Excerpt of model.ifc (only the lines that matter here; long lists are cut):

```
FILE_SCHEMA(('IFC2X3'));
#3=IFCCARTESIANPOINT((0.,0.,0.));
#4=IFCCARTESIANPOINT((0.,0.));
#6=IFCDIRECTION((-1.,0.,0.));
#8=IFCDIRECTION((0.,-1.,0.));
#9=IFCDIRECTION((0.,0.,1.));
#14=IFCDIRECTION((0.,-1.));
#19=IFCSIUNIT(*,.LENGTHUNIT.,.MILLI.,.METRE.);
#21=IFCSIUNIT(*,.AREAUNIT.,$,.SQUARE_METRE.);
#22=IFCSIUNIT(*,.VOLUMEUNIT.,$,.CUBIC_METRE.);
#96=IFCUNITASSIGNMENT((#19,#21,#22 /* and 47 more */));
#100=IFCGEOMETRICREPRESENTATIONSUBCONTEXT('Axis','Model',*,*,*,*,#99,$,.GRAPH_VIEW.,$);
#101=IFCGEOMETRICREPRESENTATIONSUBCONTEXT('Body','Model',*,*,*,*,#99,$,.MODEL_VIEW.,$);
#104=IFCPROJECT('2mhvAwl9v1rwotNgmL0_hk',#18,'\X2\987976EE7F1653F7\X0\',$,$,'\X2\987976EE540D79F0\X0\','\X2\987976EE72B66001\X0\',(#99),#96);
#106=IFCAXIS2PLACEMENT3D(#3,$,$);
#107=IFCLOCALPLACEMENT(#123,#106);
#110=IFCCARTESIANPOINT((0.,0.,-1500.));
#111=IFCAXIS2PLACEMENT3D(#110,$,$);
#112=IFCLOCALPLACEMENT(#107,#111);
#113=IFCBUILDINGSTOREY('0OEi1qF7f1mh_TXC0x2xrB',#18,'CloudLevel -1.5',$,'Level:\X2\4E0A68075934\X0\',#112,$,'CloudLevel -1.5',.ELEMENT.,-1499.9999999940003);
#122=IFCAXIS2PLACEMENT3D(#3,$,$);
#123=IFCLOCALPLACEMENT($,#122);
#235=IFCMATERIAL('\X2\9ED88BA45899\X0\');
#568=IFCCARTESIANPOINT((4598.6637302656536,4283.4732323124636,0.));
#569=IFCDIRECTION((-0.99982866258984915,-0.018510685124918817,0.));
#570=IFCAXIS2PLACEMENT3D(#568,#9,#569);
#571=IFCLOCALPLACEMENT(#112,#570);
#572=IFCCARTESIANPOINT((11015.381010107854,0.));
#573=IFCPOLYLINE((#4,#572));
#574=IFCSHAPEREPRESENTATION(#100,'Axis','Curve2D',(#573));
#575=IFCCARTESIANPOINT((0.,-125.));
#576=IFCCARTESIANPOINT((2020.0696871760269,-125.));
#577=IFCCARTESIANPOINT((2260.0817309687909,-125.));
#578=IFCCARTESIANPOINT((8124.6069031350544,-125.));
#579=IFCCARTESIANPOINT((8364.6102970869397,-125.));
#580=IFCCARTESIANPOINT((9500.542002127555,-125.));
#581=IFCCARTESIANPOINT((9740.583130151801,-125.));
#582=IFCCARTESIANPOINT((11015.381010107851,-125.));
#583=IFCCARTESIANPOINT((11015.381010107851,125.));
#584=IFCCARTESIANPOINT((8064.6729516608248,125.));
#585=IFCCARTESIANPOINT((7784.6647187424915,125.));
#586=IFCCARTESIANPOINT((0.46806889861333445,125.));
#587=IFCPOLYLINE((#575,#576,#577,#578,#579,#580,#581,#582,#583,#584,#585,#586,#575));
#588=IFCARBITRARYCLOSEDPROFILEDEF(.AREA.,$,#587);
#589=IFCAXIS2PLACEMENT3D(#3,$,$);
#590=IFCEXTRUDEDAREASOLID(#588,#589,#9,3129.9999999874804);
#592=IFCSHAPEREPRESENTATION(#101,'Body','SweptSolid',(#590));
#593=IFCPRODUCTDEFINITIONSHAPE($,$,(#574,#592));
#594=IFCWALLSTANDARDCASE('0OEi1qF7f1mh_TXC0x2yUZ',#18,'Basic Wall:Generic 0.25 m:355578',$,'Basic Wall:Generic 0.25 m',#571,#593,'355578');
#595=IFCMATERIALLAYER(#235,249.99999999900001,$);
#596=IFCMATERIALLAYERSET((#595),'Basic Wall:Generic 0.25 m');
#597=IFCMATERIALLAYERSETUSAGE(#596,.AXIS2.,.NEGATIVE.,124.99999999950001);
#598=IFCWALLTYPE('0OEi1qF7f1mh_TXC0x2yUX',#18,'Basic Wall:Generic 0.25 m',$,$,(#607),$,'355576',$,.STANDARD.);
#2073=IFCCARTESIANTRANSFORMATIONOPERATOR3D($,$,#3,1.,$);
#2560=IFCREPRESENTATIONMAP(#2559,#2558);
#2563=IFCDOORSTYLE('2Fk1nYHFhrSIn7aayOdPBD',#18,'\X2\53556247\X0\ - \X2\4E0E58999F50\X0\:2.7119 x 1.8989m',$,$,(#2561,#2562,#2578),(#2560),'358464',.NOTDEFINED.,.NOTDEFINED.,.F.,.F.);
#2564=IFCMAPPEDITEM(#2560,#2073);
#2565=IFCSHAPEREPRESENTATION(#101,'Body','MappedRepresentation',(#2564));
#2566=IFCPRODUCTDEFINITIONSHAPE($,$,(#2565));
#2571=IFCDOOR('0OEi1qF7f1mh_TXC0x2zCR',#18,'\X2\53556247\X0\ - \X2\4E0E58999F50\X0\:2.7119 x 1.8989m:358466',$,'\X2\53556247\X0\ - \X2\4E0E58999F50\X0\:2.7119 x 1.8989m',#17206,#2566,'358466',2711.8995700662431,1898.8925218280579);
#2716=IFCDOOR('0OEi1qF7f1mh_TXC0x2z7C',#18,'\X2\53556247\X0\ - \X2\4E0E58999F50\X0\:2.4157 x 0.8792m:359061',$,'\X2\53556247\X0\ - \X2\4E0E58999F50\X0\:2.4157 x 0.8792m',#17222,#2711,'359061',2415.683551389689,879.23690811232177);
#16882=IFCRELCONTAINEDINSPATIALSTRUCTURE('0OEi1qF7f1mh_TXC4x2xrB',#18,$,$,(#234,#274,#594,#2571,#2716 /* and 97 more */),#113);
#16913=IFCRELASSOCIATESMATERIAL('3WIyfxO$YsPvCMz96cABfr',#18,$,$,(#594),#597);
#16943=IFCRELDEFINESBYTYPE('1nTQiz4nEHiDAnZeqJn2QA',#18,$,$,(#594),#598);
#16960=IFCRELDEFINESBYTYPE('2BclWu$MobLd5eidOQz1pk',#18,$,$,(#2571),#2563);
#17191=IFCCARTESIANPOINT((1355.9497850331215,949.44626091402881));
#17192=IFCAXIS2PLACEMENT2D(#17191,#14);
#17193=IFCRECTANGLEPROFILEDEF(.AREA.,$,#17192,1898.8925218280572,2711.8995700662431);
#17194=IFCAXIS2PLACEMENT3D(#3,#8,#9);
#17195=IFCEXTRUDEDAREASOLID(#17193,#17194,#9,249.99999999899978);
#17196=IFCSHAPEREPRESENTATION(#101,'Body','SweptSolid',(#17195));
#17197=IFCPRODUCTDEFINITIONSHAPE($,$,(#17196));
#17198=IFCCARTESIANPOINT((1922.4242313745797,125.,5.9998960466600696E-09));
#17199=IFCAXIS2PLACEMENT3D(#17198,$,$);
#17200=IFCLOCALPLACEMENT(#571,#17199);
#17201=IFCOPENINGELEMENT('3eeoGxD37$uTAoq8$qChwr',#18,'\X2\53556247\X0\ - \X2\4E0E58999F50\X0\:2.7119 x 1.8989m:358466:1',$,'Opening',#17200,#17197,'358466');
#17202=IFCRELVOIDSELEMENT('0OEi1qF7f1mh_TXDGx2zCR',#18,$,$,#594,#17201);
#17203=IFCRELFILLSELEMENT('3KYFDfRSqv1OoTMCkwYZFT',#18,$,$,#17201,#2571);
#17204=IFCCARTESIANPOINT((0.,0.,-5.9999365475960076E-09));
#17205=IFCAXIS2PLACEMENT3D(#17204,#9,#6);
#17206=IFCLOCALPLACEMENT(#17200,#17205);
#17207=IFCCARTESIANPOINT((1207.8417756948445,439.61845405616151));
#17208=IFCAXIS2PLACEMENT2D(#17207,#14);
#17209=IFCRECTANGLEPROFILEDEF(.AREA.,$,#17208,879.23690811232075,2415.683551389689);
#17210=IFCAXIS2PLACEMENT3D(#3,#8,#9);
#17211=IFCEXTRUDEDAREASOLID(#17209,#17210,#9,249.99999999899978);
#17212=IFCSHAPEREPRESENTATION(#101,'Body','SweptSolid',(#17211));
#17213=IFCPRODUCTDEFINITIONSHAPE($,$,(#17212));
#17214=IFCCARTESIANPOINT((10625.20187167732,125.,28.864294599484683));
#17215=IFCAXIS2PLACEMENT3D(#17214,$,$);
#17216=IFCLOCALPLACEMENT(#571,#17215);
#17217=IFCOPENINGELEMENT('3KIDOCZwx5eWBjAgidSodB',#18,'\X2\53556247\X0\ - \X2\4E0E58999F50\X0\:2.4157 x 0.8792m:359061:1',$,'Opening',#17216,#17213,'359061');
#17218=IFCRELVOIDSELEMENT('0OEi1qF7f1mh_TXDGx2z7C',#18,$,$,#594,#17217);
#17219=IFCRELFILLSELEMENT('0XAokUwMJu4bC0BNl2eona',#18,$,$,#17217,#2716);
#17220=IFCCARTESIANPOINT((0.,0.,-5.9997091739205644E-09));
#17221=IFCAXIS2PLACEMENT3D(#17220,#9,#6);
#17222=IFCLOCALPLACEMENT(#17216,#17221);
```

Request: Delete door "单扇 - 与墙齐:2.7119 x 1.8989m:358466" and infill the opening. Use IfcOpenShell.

```python
import ifcopenshell
import ifcopenshell.api.feature
import ifcopenshell.api.root
import ifcopenshell.geom
import ifcopenshell.util.shape

model = ifcopenshell.open("model.ifc")
settings = ifcopenshell.geom.settings()


def volume(element):
    """Net volume in cubic metres, openings subtracted."""
    shape = ifcopenshell.geom.create_shape(settings, element)
    return ifcopenshell.util.shape.get_volume(shape.geometry)


door = model.by_guid("0OEi1qF7f1mh_TXC0x2zCR")
opening = door.FillsVoids[0].RelatingOpeningElement
wall = opening.VoidsElements[0].RelatingBuildingElement
before = volume(wall)

ifcopenshell.api.root.remove_product(model, product=door)
ifcopenshell.api.feature.remove_feature(model, feature=opening)

after = volume(wall)

print(f"wall volume {before:.3f} -> {after:.3f} m3")

model.write("model-out.ifc")
```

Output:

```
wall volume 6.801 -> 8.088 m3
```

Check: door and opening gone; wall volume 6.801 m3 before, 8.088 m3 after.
